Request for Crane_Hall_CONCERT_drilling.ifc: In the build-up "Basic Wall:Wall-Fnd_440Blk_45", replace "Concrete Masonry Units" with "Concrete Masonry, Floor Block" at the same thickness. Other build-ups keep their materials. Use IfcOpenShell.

First a look at what the model holds.

```python
import ifcopenshell
import ifcopenshell.util.element

model = ifcopenshell.open("Crane_Hall_CONCERT_drilling.ifc")
print(model.schema)
for layer_set in model.by_type("IfcMaterialLayerSet"):
    if layer_set.LayerSetName == "Basic Wall:Wall-Fnd_440Blk_45":
        for layer in layer_set.MaterialLayers:
            print(layer.id(), layer.Material and layer.Material.Name, layer.LayerThickness, sep=" | ")
        print(len(ifcopenshell.util.element.get_elements_by_material(model, layer_set)), "elements and types use it")
print(sorted(m.Name for m in model.by_type("IfcMaterial") if m.Name)[:60])
```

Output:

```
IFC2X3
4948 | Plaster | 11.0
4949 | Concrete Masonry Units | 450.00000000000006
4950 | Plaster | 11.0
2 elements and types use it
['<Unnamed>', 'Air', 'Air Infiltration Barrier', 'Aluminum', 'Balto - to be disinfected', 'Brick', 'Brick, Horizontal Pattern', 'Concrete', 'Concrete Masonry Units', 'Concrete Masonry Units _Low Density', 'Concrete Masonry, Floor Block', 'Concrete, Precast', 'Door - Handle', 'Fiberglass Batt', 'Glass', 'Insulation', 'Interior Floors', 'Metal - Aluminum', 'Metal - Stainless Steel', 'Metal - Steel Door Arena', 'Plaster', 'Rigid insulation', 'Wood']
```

```python
import ifcopenshell
import ifcopenshell.api.material

model = ifcopenshell.open("Crane_Hall_CONCERT_drilling.ifc")

layer_set = next(s for s in model.by_type("IfcMaterialLayerSet") if s.LayerSetName == "Basic Wall:Wall-Fnd_440Blk_45")
layer = next(l for l in layer_set.MaterialLayers if l.Material and l.Material.Name == "Concrete Masonry Units")
material = next(m for m in model.by_type("IfcMaterial") if m.Name == "Concrete Masonry, Floor Block")

# Point this one layer at the other material; renaming the old one would change it everywhere.
ifcopenshell.api.material.edit_layer(model, layer=layer, attributes={}, material=material)

print([l.Material.Name if l.Material else None for l in layer_set.MaterialLayers])

model.write("Crane_Hall_CONCERT_drilling_edited.ifc")
```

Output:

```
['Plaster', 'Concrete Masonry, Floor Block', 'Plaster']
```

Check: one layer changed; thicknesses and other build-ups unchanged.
